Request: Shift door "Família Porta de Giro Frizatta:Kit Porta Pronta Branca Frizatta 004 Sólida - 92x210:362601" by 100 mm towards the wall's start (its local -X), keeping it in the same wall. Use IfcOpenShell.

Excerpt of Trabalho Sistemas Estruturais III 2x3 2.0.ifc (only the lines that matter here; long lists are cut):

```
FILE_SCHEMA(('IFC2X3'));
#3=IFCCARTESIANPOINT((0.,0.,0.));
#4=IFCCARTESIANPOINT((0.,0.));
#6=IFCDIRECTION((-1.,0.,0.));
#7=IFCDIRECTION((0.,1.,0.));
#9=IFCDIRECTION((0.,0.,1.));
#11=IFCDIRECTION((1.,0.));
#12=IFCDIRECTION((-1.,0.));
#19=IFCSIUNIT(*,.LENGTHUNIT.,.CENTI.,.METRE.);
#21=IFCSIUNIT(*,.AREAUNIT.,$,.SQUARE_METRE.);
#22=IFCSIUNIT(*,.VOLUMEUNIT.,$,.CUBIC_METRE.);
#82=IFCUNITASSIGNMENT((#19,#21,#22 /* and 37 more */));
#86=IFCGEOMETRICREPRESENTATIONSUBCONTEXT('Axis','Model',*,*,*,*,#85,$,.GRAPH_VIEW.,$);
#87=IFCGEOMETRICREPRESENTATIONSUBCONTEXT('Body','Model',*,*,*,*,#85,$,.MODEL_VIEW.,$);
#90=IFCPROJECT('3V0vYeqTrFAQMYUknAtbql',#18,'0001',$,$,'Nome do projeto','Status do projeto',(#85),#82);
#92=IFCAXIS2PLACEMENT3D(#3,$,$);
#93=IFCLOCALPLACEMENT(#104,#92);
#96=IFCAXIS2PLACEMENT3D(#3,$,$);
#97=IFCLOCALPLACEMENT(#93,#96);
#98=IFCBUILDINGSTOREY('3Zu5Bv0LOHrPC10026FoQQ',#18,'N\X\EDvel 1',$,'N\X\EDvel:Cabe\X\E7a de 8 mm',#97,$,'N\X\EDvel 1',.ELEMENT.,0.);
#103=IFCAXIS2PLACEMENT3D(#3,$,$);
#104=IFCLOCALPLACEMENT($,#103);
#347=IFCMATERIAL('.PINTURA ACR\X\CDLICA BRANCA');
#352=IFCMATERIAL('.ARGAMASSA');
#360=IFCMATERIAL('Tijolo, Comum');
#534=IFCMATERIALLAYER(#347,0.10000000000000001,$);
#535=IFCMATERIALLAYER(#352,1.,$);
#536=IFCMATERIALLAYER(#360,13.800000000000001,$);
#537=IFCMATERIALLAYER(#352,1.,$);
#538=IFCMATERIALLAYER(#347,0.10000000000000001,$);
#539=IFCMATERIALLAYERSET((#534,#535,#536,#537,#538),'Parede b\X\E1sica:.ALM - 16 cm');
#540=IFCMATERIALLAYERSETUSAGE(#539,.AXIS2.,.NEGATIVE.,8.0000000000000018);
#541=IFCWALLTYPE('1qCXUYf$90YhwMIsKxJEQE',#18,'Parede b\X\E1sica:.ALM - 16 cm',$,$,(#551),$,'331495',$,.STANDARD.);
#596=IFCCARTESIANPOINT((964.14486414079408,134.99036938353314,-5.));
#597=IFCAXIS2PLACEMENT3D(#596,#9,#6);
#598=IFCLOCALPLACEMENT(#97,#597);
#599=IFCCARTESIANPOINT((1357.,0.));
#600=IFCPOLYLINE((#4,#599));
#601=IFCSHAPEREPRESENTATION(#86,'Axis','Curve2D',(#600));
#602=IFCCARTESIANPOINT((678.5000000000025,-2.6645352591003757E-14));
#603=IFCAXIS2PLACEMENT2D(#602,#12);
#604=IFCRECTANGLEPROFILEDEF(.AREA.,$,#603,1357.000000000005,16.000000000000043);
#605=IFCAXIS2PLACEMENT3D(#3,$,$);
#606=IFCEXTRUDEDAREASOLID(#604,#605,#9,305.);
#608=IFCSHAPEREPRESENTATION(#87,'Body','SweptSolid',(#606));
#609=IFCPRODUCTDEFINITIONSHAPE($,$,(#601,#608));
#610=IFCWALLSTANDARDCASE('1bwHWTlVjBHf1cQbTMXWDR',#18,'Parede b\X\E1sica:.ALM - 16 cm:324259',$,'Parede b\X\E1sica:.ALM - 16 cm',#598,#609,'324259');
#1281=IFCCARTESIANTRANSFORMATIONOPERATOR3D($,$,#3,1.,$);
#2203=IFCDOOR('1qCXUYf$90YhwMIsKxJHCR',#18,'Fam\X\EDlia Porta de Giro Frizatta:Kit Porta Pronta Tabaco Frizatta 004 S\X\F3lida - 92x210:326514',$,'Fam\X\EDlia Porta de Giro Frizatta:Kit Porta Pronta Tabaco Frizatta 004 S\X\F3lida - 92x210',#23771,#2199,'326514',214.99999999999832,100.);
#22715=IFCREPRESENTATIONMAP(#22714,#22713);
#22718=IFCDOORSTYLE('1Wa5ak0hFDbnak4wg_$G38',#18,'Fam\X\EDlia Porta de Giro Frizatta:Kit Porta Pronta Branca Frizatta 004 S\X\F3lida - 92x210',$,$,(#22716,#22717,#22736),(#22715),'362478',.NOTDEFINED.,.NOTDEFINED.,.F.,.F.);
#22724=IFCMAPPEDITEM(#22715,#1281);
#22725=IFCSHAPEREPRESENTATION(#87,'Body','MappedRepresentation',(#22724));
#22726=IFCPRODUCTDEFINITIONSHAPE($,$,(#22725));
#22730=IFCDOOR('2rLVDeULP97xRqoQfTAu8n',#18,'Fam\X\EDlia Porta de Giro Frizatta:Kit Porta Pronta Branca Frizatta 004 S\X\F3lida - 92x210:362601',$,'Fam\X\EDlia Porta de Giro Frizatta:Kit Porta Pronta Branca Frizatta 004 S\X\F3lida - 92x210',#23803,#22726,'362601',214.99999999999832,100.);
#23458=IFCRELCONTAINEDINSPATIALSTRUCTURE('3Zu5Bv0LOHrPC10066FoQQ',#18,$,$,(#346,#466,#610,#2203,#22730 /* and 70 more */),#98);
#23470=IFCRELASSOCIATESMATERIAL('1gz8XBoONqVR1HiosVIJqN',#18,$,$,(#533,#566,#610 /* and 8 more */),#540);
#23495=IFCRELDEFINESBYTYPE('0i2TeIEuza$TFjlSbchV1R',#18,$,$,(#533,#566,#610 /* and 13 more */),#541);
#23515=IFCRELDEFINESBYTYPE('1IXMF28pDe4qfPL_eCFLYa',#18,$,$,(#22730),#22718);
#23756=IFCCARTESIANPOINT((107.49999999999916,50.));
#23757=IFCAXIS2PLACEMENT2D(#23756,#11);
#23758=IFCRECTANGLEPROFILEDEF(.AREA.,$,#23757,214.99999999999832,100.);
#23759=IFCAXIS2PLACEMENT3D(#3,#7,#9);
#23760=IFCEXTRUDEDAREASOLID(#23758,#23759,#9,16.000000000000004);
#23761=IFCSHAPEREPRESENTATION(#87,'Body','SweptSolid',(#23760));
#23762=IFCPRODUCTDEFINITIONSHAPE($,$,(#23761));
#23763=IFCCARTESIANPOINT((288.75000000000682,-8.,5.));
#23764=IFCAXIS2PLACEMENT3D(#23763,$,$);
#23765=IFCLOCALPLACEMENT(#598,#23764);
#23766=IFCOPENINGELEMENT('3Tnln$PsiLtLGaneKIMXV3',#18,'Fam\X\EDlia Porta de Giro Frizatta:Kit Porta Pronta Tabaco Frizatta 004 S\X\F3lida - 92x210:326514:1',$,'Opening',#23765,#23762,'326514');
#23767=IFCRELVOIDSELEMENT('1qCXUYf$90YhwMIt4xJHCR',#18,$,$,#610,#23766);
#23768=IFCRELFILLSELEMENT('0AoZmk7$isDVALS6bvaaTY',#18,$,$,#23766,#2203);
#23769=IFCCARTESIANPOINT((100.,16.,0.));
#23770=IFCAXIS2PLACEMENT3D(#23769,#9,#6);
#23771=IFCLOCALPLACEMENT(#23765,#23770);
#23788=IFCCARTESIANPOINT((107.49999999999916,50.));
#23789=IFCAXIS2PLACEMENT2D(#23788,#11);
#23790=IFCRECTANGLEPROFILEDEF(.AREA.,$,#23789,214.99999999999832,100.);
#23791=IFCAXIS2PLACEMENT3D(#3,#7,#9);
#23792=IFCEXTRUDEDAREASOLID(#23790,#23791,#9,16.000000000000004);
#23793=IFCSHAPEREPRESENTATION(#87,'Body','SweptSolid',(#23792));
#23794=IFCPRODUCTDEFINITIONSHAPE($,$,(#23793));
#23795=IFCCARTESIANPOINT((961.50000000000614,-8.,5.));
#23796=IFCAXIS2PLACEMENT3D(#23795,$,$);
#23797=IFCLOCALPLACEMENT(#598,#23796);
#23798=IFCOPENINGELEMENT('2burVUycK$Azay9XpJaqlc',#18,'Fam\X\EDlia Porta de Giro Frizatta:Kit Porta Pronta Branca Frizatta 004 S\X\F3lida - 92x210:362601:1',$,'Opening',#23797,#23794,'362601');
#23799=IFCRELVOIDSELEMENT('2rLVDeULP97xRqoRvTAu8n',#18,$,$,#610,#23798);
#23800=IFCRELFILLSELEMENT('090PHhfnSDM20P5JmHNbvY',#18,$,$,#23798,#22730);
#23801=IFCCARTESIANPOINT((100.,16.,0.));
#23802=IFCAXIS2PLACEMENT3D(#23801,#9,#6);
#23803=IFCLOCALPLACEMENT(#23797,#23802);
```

```python
import ifcopenshell
import ifcopenshell.api.geometry
import ifcopenshell.util.placement
import ifcopenshell.util.unit

model = ifcopenshell.open("Trabalho Sistemas Estruturais III 2x3 2.0.ifc")
unit_scale = ifcopenshell.util.unit.calculate_unit_scale(model)

door = model.by_guid("2rLVDeULP97xRqoQfTAu8n")
opening = door.FillsVoids[0].RelatingOpeningElement
wall = opening.VoidsElements[0].RelatingBuildingElement

wall_matrix = ifcopenshell.util.placement.get_local_placement(wall.ObjectPlacement)
shift = wall_matrix[:3, 0] * -0.1 / unit_scale
before = ifcopenshell.util.placement.get_local_placement(door.ObjectPlacement)[:3, 3].copy()

# The door is placed relative to its opening, so it follows when the opening moves.
matrix = ifcopenshell.util.placement.get_local_placement(opening.ObjectPlacement)
matrix[:3, 3] += shift
ifcopenshell.api.geometry.edit_object_placement(
    model, product=opening, matrix=matrix, is_si=False, should_transform_children=True
)

after = ifcopenshell.util.placement.get_local_placement(door.ObjectPlacement)[:3, 3]
print("door moved by", (after - before).round(3) + 0.0)

model.write("Trabalho Sistemas Estruturais III 2x3 2.0_rev.ifc")
```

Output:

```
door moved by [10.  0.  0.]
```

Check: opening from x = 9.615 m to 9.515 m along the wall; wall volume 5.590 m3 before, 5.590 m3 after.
